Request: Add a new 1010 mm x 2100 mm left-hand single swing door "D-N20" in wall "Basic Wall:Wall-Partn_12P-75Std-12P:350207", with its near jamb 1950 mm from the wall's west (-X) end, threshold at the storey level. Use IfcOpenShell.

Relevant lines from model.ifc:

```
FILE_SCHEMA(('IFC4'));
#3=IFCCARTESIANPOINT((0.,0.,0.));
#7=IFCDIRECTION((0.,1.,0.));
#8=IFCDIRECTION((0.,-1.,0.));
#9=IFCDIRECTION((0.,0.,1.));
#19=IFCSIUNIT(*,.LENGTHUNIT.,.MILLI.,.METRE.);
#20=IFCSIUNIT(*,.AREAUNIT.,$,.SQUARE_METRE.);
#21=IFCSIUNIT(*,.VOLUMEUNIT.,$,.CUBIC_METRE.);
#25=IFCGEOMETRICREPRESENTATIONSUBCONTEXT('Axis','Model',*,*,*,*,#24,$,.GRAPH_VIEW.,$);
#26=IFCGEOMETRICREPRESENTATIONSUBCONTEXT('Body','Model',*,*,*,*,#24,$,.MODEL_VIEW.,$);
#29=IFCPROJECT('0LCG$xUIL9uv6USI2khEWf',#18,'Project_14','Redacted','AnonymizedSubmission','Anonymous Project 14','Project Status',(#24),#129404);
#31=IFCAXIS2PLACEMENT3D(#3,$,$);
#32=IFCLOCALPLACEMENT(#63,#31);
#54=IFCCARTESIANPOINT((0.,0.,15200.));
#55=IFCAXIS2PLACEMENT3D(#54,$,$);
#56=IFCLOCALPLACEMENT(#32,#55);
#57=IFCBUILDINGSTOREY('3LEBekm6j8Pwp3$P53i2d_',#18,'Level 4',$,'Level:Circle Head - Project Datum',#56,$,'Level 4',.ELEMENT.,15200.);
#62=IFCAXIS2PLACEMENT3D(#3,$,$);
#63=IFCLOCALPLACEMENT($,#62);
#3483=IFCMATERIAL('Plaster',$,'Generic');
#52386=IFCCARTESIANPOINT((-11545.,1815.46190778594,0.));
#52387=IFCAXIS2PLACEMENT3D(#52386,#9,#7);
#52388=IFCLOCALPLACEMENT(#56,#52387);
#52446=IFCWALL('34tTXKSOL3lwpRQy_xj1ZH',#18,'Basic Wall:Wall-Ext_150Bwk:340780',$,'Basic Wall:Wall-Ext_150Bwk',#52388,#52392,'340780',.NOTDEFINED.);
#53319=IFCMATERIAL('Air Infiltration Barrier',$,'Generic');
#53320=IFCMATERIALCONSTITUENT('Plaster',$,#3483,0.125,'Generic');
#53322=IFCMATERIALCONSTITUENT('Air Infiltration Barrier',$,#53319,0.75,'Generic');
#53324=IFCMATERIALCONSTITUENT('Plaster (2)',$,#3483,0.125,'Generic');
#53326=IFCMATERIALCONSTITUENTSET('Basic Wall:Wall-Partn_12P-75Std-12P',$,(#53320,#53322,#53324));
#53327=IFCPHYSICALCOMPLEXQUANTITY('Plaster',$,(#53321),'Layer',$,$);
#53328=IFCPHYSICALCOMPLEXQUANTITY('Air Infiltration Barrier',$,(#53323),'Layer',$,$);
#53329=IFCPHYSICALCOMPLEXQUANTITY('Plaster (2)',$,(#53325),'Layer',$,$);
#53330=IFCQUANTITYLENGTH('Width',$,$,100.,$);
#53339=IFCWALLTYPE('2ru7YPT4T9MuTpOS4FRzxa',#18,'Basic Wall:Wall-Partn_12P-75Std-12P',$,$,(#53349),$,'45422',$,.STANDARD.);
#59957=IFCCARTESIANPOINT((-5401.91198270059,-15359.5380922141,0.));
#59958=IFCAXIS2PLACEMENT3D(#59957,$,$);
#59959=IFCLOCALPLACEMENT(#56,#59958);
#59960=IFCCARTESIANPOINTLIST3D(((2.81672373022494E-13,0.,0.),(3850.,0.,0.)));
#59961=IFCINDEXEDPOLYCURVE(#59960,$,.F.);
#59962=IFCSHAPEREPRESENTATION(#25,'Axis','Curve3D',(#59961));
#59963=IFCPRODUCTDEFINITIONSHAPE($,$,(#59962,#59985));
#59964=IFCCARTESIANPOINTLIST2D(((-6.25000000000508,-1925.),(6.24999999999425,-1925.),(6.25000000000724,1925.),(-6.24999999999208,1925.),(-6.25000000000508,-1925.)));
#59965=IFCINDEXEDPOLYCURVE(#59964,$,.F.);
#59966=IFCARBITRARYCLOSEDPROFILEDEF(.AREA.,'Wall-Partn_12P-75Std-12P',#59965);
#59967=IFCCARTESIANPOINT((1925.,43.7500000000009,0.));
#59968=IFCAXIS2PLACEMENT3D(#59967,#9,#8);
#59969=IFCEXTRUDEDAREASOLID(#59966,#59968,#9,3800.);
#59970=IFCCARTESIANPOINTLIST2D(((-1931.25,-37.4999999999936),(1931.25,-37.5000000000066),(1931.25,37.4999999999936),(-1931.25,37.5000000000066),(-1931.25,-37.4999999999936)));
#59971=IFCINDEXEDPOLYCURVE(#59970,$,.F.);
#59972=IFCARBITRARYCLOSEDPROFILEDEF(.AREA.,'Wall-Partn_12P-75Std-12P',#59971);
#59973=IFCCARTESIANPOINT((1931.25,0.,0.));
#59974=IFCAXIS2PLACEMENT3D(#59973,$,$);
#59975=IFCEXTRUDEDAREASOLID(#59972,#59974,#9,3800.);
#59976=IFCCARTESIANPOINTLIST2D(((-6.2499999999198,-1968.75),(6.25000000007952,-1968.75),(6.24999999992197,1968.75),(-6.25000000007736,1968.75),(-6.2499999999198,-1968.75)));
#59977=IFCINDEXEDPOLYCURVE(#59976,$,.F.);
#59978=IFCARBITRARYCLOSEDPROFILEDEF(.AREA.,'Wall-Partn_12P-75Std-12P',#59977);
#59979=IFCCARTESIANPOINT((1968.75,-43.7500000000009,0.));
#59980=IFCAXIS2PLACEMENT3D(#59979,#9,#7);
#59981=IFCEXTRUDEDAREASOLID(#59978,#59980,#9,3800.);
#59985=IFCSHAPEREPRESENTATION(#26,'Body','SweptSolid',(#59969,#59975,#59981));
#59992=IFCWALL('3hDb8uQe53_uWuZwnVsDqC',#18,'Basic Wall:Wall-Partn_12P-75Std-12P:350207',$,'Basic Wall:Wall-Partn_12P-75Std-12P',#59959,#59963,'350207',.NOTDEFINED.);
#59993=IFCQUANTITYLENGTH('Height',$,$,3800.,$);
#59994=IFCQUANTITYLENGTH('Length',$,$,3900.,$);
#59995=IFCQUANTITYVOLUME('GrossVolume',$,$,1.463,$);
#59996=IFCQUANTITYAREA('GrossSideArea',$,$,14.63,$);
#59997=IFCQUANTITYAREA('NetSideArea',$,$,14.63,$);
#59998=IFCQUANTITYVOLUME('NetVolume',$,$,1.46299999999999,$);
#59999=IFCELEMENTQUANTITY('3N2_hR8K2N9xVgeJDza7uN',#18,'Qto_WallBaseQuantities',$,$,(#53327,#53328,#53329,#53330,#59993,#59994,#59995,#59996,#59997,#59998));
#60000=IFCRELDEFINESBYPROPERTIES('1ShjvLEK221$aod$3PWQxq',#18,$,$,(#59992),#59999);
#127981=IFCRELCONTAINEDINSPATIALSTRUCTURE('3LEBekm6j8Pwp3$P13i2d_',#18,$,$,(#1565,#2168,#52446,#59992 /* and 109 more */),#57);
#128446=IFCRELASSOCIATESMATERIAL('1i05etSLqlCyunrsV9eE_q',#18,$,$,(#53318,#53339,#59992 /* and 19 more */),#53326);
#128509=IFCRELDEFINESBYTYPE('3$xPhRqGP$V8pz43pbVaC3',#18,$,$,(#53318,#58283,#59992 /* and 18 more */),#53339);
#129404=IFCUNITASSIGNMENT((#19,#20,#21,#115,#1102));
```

```python
import numpy as np
import ifcopenshell
import ifcopenshell.api.feature
import ifcopenshell.api.geometry
import ifcopenshell.api.pset
import ifcopenshell.api.root
import ifcopenshell.api.spatial
import ifcopenshell.geom
import ifcopenshell.util.element
import ifcopenshell.util.placement
import ifcopenshell.util.representation
import ifcopenshell.util.shape
import ifcopenshell.util.unit

model = ifcopenshell.open("model.ifc")
unit_scale = ifcopenshell.util.unit.calculate_unit_scale(model)
area_scale = ifcopenshell.util.unit.calculate_unit_scale(model, "AREAUNIT")
volume_scale = ifcopenshell.util.unit.calculate_unit_scale(model, "VOLUMEUNIT")
settings = ifcopenshell.geom.settings()


def volume(element):
    """Net volume in cubic metres, openings subtracted."""
    shape = ifcopenshell.geom.create_shape(settings, element)
    return ifcopenshell.util.shape.get_volume(shape.geometry)


wall = model.by_id(59992)
storey = ifcopenshell.util.element.get_container(wall, ifc_class="IfcBuildingStorey")
context = ifcopenshell.util.representation.get_context(model, "Model", "Body", "MODEL_VIEW")
before = volume(wall)

width, height, from_end, sill = 1.01, 2.1, 1.95, 0.0  # metres

# The wall runs along its own X axis, and the end named is its -X end.
wall_shape = ifcopenshell.geom.create_shape(settings, wall)
x, y, z = ifcopenshell.util.shape.get_vertices(wall_shape.geometry).T
start = x.min() + from_end
face, thickness = float(y.min()), float(y.max() - y.min())
wall_matrix = ifcopenshell.util.placement.get_local_placement(wall.ObjectPlacement)
level = ifcopenshell.util.placement.get_local_placement(storey.ObjectPlacement)[2, 3]


def in_wall(x, y):
    """Placement at x, y metres in the wall's axes, at sill height."""
    matrix = wall_matrix.copy()
    matrix[:, 3] = wall_matrix @ np.array([x / unit_scale, y / unit_scale, 0.0, 1.0])
    matrix[2, 3] = level + sill / unit_scale
    return matrix


# Opening: a box that overshoots both wall faces by 50 mm.
opening = ifcopenshell.api.root.create_entity(model, ifc_class="IfcOpeningElement", predefined_type="OPENING")
box = ifcopenshell.api.geometry.add_wall_representation(
    model, context=context, length=width, height=height, thickness=thickness + 0.1
)
ifcopenshell.api.geometry.assign_representation(model, product=opening, representation=box)
ifcopenshell.api.geometry.edit_object_placement(model, product=opening, matrix=in_wall(start, face - 0.05), is_si=False)
ifcopenshell.api.feature.add_feature(model, feature=opening, element=wall)

door = ifcopenshell.api.root.create_entity(model, ifc_class="IfcDoor", name="D-N20", predefined_type="DOOR")
door.OverallWidth, door.OverallHeight = width / unit_scale, height / unit_scale
door.OperationType = "SINGLE_SWING_LEFT"
body = ifcopenshell.api.geometry.add_door_representation(
    model,
    context=context,
    overall_width=door.OverallWidth,
    overall_height=door.OverallHeight,
    operation_type="SINGLE_SWING_LEFT",
    lining_properties={"LiningDepth": thickness / unit_scale, "ThresholdDepth": thickness / unit_scale},
)
ifcopenshell.api.geometry.assign_representation(model, product=door, representation=body)
ifcopenshell.api.spatial.assign_container(model, products=[door], relating_structure=storey)
ifcopenshell.api.feature.add_filling(model, opening=opening, element=door)

# The lining spans the wall, so the door starts at the wall face.
ifcopenshell.api.geometry.edit_object_placement(model, product=door, matrix=in_wall(start, face), is_si=False)

after = volume(wall)

# Update the wall's stored quantities.
qto = model.by_id(ifcopenshell.util.element.get_pset(wall, "Qto_WallBaseQuantities", should_inherit=False)["id"])
ifcopenshell.api.pset.edit_qto(model, qto=qto, properties={
    "NetSideArea": after / thickness / area_scale,
    "NetVolume": after / volume_scale,
})

print(f"wall volume {before:.3f} -> {after:.3f} m3")

model.write("model_v2.ifc")
```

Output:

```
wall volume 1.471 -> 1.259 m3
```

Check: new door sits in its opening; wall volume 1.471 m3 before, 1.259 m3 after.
